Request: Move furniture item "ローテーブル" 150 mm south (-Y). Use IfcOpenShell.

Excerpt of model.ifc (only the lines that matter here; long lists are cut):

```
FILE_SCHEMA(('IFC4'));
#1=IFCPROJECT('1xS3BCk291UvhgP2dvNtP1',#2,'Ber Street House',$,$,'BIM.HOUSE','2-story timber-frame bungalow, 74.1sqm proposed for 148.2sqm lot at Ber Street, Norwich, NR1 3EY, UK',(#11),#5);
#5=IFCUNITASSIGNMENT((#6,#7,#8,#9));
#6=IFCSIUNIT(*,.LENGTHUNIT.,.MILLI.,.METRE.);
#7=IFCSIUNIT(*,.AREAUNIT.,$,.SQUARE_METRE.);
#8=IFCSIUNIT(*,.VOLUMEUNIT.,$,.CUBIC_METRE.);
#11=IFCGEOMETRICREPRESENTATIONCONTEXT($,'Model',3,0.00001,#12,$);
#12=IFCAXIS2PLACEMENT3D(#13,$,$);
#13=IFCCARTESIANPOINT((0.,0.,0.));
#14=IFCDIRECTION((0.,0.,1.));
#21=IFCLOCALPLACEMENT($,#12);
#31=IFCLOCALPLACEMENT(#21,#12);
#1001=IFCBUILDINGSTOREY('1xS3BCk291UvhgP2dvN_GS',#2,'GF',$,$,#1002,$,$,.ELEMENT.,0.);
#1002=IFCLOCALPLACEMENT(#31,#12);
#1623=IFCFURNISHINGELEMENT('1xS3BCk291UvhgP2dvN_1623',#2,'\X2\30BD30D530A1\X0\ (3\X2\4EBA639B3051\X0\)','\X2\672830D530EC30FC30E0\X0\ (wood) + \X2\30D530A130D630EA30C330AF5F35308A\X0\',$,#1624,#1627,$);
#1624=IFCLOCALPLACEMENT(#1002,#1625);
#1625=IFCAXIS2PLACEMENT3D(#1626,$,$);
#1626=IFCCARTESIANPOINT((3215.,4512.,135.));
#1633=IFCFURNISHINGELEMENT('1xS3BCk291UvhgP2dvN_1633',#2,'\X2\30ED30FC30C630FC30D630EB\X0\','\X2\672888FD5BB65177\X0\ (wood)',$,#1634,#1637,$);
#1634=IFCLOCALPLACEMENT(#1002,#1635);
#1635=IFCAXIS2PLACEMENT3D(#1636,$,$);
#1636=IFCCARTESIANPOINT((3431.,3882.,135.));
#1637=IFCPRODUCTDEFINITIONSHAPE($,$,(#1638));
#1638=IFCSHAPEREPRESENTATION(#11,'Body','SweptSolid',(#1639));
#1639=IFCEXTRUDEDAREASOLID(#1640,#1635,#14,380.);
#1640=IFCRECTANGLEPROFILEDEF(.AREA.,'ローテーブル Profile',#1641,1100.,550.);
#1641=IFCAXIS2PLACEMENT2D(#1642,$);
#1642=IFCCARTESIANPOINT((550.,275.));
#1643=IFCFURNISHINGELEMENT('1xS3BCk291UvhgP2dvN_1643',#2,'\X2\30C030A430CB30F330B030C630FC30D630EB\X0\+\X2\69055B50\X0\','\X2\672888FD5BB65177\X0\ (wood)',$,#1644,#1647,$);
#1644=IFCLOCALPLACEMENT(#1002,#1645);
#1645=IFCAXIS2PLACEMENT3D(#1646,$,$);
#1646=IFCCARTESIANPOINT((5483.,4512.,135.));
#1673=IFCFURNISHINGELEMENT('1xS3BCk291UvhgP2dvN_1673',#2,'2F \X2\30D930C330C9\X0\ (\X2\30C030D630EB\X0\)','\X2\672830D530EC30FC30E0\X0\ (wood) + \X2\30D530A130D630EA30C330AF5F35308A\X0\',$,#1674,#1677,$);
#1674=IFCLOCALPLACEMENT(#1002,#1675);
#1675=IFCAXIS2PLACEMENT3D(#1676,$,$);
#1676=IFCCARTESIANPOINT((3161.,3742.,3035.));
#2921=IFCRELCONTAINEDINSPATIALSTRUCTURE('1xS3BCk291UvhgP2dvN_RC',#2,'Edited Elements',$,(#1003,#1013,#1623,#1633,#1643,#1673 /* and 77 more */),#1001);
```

```python
import ifcopenshell
import ifcopenshell.api.geometry
import ifcopenshell.util.placement

model = ifcopenshell.open("model.ifc")

item = model.by_guid("1xS3BCk291UvhgP2dvN_1633")
matrix = ifcopenshell.util.placement.get_local_placement(item.ObjectPlacement)
matrix[1, 3] -= 150.0
ifcopenshell.api.geometry.edit_object_placement(model, product=item, matrix=matrix, is_si=False)

print(ifcopenshell.util.placement.get_local_placement(item.ObjectPlacement).round(3) + 0.0)

model.write("model_v2.ifc")
```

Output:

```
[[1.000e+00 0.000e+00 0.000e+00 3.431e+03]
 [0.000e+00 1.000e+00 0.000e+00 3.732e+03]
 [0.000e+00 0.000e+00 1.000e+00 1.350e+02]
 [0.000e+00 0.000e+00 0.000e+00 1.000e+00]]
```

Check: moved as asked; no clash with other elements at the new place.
